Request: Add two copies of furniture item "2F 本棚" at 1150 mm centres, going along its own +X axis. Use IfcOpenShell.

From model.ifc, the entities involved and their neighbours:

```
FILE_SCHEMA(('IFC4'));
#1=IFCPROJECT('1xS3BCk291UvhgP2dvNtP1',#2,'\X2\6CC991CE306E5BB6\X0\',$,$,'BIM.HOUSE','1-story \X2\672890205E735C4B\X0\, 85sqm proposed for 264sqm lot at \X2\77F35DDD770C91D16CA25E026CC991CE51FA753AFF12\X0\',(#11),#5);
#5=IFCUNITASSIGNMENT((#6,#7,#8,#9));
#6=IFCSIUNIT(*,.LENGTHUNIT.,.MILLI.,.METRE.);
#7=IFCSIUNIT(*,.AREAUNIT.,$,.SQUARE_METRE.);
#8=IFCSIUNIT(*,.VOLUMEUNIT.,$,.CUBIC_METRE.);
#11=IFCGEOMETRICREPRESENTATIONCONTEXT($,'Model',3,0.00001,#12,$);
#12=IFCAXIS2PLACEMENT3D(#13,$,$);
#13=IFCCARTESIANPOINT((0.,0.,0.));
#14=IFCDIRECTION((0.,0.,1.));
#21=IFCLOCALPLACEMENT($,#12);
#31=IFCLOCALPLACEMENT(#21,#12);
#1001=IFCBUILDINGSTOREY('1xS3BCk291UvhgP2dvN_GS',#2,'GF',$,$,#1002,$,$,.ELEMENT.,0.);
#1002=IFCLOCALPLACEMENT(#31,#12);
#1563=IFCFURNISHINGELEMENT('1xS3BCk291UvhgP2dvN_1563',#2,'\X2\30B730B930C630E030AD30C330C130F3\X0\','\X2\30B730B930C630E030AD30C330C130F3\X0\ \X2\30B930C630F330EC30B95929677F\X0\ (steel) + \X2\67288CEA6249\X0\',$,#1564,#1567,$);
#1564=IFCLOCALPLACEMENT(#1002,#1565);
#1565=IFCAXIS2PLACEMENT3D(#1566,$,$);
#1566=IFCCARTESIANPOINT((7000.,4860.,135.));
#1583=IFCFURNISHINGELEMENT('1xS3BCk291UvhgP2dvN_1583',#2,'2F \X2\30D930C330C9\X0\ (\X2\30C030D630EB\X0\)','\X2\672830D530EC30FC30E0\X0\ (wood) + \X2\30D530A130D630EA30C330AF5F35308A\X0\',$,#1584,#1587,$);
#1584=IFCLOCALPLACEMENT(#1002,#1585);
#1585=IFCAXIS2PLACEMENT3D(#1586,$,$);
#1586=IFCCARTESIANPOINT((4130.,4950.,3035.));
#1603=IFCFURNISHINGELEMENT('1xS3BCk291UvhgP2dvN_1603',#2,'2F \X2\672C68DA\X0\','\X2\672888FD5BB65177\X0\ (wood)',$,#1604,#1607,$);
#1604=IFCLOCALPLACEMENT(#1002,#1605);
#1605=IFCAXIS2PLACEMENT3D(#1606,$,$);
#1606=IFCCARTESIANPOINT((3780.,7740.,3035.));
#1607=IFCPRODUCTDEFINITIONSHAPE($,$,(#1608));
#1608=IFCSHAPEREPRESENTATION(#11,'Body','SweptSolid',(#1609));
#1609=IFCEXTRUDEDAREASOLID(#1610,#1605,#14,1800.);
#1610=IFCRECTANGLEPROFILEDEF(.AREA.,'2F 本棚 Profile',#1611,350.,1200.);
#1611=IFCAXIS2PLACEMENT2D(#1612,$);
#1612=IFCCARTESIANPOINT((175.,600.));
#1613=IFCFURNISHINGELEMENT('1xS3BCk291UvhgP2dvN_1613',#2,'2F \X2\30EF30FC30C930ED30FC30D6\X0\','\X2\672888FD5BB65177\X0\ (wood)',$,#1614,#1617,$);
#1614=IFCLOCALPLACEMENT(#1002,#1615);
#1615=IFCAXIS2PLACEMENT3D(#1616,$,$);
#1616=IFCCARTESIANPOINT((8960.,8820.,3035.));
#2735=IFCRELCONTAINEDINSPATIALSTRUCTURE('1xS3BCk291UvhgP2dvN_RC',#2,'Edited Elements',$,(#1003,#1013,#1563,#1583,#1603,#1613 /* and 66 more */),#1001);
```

```python
import ifcopenshell
import ifcopenshell.api.geometry
import ifcopenshell.api.root
import ifcopenshell.util.element
import ifcopenshell.util.placement
import ifcopenshell.util.unit

model = ifcopenshell.open("model.ifc")
unit_scale = ifcopenshell.util.unit.calculate_unit_scale(model)


def reuse_history(source, copy):
    """copy_class also copies each property set's owner history, people and application; keep the originals."""
    for rel in copy.IsDefinedBy:
        if rel.is_a("IfcRelDefinesByProperties") and (history := rel.RelatingPropertyDefinition.OwnerHistory):
            rel.RelatingPropertyDefinition.OwnerHistory = source.OwnerHistory
            ifcopenshell.util.element.remove_deep2(model, history)


source = model.by_guid("1xS3BCk291UvhgP2dvN_1603")
base = ifcopenshell.util.placement.get_local_placement(source.ObjectPlacement)
step = base[:3, 0] * 1.15 / unit_scale

for i in range(1, 3):
    copy = ifcopenshell.api.root.copy_class(model, product=source)
    copy.Representation = ifcopenshell.util.element.copy_deep(
        model, source.Representation, exclude=["IfcGeometricRepresentationContext", "IfcRepresentationMap"]
    )
    reuse_history(source, copy)
    matrix = base.copy()
    matrix[:3, 3] += i * step
    print("added at", matrix[:3, 3].round(3) + 0.0)
    ifcopenshell.api.geometry.edit_object_placement(model, product=copy, matrix=matrix, is_si=False)

model.write("model_v2.ifc")
```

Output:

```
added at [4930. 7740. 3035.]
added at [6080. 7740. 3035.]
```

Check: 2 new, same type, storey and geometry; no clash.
